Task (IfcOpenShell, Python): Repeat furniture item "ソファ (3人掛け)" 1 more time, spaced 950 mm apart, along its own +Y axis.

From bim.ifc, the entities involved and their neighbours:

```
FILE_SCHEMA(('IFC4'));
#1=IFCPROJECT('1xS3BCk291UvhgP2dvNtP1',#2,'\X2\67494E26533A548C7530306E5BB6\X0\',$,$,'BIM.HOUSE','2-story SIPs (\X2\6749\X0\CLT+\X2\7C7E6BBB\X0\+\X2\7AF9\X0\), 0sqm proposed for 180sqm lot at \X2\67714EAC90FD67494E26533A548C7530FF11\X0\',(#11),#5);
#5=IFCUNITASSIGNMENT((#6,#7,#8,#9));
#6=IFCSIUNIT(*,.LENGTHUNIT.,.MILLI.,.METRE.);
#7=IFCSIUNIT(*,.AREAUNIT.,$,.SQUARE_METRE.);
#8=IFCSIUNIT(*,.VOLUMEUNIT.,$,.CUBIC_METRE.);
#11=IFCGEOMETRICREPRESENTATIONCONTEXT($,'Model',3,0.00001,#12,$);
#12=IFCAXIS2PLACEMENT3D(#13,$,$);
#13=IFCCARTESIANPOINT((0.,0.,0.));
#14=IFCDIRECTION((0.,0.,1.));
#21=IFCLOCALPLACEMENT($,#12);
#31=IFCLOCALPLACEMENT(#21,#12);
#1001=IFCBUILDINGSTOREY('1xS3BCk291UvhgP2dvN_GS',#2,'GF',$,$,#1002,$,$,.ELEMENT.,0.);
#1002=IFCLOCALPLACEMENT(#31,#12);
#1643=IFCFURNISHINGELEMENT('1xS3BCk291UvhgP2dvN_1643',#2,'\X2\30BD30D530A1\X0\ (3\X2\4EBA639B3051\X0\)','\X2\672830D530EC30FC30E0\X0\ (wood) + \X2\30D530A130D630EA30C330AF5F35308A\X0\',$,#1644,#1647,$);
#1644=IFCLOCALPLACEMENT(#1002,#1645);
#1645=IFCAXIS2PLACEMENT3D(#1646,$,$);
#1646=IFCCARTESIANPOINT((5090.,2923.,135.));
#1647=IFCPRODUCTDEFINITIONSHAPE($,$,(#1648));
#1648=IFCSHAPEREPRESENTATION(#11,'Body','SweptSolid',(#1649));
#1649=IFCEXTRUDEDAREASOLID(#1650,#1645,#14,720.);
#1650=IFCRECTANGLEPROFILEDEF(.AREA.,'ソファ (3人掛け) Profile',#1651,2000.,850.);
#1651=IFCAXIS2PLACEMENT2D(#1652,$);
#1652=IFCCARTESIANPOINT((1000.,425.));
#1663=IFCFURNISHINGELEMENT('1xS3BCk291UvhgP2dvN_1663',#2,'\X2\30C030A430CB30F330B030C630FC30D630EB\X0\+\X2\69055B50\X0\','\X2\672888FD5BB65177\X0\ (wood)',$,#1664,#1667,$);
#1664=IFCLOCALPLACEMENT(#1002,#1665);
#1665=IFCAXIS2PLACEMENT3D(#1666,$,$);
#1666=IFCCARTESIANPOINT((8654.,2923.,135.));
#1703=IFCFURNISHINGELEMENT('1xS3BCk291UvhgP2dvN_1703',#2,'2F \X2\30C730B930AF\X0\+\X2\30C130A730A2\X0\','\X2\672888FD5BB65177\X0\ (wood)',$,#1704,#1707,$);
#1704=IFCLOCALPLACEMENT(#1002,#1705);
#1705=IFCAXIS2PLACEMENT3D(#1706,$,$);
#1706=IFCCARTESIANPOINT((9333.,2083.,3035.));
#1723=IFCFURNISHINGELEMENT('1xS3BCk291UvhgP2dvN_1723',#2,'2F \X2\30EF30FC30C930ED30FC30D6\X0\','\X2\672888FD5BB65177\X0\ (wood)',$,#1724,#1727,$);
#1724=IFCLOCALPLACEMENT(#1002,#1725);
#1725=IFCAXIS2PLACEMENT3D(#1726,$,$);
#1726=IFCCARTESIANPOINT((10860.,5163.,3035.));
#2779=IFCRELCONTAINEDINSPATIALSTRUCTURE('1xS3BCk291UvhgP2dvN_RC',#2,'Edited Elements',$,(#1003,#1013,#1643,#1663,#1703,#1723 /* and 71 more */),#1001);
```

```python
import ifcopenshell
import ifcopenshell.api.geometry
import ifcopenshell.api.root
import ifcopenshell.util.element
import ifcopenshell.util.placement

model = ifcopenshell.open("bim.ifc")


def reuse_history(source, copy):
    """copy_class also copies each property set's owner history, people and application; keep the originals."""
    for rel in copy.IsDefinedBy:
        if rel.is_a("IfcRelDefinesByProperties") and (history := rel.RelatingPropertyDefinition.OwnerHistory):
            rel.RelatingPropertyDefinition.OwnerHistory = source.OwnerHistory
            ifcopenshell.util.element.remove_deep2(model, history)


source = model.by_id(1643)
base = ifcopenshell.util.placement.get_local_placement(source.ObjectPlacement)
step = base[:3, 1] * 950.0

for i in range(1, 2):
    copy = ifcopenshell.api.root.copy_class(model, product=source)
    copy.Representation = ifcopenshell.util.element.copy_deep(
        model, source.Representation, exclude=["IfcGeometricRepresentationContext", "IfcRepresentationMap"]
    )
    reuse_history(source, copy)
    matrix = base.copy()
    matrix[:3, 3] += i * step
    print("added at", matrix[:3, 3].round(3) + 0.0)
    ifcopenshell.api.geometry.edit_object_placement(model, product=copy, matrix=matrix, is_si=False)

model.write("bim_edited.ifc")
```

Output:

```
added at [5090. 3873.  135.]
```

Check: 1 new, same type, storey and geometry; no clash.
